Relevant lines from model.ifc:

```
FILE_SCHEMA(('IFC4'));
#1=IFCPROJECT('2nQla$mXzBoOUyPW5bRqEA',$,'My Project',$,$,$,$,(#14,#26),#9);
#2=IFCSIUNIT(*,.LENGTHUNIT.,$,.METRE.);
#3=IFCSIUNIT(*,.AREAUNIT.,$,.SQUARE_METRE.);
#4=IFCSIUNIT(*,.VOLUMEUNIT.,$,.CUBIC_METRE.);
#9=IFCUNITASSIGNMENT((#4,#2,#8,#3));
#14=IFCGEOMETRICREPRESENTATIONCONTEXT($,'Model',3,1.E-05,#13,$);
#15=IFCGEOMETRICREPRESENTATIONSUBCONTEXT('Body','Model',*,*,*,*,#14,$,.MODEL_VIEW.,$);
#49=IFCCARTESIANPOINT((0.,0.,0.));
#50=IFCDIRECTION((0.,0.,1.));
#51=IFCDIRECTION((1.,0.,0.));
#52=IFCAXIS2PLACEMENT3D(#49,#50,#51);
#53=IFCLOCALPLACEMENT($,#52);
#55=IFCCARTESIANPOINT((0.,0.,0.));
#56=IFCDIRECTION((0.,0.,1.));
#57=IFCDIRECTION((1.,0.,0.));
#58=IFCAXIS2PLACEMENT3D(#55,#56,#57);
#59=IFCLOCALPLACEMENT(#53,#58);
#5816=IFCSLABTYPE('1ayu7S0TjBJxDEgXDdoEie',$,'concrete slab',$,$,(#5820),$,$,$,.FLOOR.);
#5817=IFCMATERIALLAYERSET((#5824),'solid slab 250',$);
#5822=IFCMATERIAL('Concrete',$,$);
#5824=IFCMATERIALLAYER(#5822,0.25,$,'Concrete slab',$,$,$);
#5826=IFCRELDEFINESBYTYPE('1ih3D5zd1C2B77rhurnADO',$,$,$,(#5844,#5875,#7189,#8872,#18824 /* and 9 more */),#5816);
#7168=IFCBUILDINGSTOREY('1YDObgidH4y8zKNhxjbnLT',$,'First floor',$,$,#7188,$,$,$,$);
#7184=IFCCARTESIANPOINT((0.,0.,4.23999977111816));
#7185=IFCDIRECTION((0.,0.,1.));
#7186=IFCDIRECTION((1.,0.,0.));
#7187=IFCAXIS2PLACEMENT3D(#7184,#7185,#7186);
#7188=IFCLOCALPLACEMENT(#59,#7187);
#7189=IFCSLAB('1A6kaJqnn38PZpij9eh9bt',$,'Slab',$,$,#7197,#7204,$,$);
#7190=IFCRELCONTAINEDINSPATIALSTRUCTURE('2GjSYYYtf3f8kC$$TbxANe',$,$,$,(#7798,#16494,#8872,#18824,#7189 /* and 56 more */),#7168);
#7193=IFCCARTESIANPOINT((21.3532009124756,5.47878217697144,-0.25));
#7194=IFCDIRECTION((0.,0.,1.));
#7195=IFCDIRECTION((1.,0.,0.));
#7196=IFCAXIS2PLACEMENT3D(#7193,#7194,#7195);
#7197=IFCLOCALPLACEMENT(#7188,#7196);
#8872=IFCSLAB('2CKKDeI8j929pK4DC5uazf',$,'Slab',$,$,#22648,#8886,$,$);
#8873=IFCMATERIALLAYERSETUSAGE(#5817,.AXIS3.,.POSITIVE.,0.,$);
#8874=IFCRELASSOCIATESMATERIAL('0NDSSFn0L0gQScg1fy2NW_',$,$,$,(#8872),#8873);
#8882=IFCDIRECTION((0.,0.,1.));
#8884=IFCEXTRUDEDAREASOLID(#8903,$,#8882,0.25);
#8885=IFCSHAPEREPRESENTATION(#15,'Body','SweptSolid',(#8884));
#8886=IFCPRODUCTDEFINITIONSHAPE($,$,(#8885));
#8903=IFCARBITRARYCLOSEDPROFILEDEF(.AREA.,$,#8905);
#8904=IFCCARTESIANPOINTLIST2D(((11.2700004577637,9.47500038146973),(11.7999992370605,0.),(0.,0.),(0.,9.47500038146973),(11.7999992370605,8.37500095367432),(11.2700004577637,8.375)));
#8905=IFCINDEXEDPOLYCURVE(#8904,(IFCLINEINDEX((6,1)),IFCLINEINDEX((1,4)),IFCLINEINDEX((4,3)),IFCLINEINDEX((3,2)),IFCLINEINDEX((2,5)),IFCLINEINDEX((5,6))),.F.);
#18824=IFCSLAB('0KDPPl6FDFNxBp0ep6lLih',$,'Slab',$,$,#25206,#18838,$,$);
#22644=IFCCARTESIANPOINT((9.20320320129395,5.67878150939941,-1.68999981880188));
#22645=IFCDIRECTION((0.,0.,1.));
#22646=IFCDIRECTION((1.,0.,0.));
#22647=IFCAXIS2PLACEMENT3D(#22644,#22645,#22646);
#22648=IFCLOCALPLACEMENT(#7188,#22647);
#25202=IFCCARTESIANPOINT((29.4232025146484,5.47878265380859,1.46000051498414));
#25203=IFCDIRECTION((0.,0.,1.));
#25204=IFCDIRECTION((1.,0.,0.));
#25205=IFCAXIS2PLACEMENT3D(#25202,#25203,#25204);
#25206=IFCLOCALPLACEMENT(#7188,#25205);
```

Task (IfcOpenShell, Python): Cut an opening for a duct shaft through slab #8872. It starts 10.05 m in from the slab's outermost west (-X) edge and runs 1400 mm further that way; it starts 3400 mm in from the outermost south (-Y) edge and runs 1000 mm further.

```python
import numpy as np
import ifcopenshell
import ifcopenshell.api.feature
import ifcopenshell.api.geometry
import ifcopenshell.api.root
import ifcopenshell.geom
import ifcopenshell.util.placement
import ifcopenshell.util.representation
import ifcopenshell.util.shape
import ifcopenshell.util.unit

model = ifcopenshell.open("model.ifc")
unit_scale = ifcopenshell.util.unit.calculate_unit_scale(model)
settings = ifcopenshell.geom.settings()


def volume(element):
    """Net volume in cubic metres, openings subtracted."""
    shape = ifcopenshell.geom.create_shape(settings, element)
    return ifcopenshell.util.shape.get_volume(shape.geometry)


slab = model.by_guid("2CKKDeI8j929pK4DC5uazf")
before = volume(slab)

# Extent in the slab's own axes, in metres. The edges named are its -X and -Y sides.
slab_shape = ifcopenshell.geom.create_shape(settings, slab)
vertices = ifcopenshell.util.shape.get_vertices(slab_shape.geometry)
x_min, y_min, bottom = vertices.min(axis=0)
top = vertices[:, 2].max()

opening = ifcopenshell.api.root.create_entity(model, ifc_class="IfcOpeningElement", name="Duct shaft opening", predefined_type="OPENING")
context = ifcopenshell.util.representation.get_context(model, "Model", "Body", "MODEL_VIEW")
width, depth = 1.4, 1
outline = [(0.0, 0.0), (width, 0.0), (width, depth), (0.0, depth), (0.0, 0.0)]
# Overshoot both faces by 50 mm so the cut is clean.
shape = ifcopenshell.api.geometry.add_slab_representation(
    model, context=context, depth=top - bottom + 0.1, polyline=outline
)
ifcopenshell.api.geometry.assign_representation(model, product=opening, representation=shape)

matrix = ifcopenshell.util.placement.get_local_placement(slab.ObjectPlacement)
matrix[:, 3] = matrix @ np.append(np.array([x_min + 10.05, y_min + 3.4, bottom - 0.05]) / unit_scale, 1.0)
ifcopenshell.api.geometry.edit_object_placement(model, product=opening, matrix=matrix, is_si=False)
ifcopenshell.api.feature.add_feature(model, feature=opening, element=slab)

after = volume(slab)

print(f"slab volume {before:.3f} -> {after:.3f} m3")

model.write("model_v2.ifc")
```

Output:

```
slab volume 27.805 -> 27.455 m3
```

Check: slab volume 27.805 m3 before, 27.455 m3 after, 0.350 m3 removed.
